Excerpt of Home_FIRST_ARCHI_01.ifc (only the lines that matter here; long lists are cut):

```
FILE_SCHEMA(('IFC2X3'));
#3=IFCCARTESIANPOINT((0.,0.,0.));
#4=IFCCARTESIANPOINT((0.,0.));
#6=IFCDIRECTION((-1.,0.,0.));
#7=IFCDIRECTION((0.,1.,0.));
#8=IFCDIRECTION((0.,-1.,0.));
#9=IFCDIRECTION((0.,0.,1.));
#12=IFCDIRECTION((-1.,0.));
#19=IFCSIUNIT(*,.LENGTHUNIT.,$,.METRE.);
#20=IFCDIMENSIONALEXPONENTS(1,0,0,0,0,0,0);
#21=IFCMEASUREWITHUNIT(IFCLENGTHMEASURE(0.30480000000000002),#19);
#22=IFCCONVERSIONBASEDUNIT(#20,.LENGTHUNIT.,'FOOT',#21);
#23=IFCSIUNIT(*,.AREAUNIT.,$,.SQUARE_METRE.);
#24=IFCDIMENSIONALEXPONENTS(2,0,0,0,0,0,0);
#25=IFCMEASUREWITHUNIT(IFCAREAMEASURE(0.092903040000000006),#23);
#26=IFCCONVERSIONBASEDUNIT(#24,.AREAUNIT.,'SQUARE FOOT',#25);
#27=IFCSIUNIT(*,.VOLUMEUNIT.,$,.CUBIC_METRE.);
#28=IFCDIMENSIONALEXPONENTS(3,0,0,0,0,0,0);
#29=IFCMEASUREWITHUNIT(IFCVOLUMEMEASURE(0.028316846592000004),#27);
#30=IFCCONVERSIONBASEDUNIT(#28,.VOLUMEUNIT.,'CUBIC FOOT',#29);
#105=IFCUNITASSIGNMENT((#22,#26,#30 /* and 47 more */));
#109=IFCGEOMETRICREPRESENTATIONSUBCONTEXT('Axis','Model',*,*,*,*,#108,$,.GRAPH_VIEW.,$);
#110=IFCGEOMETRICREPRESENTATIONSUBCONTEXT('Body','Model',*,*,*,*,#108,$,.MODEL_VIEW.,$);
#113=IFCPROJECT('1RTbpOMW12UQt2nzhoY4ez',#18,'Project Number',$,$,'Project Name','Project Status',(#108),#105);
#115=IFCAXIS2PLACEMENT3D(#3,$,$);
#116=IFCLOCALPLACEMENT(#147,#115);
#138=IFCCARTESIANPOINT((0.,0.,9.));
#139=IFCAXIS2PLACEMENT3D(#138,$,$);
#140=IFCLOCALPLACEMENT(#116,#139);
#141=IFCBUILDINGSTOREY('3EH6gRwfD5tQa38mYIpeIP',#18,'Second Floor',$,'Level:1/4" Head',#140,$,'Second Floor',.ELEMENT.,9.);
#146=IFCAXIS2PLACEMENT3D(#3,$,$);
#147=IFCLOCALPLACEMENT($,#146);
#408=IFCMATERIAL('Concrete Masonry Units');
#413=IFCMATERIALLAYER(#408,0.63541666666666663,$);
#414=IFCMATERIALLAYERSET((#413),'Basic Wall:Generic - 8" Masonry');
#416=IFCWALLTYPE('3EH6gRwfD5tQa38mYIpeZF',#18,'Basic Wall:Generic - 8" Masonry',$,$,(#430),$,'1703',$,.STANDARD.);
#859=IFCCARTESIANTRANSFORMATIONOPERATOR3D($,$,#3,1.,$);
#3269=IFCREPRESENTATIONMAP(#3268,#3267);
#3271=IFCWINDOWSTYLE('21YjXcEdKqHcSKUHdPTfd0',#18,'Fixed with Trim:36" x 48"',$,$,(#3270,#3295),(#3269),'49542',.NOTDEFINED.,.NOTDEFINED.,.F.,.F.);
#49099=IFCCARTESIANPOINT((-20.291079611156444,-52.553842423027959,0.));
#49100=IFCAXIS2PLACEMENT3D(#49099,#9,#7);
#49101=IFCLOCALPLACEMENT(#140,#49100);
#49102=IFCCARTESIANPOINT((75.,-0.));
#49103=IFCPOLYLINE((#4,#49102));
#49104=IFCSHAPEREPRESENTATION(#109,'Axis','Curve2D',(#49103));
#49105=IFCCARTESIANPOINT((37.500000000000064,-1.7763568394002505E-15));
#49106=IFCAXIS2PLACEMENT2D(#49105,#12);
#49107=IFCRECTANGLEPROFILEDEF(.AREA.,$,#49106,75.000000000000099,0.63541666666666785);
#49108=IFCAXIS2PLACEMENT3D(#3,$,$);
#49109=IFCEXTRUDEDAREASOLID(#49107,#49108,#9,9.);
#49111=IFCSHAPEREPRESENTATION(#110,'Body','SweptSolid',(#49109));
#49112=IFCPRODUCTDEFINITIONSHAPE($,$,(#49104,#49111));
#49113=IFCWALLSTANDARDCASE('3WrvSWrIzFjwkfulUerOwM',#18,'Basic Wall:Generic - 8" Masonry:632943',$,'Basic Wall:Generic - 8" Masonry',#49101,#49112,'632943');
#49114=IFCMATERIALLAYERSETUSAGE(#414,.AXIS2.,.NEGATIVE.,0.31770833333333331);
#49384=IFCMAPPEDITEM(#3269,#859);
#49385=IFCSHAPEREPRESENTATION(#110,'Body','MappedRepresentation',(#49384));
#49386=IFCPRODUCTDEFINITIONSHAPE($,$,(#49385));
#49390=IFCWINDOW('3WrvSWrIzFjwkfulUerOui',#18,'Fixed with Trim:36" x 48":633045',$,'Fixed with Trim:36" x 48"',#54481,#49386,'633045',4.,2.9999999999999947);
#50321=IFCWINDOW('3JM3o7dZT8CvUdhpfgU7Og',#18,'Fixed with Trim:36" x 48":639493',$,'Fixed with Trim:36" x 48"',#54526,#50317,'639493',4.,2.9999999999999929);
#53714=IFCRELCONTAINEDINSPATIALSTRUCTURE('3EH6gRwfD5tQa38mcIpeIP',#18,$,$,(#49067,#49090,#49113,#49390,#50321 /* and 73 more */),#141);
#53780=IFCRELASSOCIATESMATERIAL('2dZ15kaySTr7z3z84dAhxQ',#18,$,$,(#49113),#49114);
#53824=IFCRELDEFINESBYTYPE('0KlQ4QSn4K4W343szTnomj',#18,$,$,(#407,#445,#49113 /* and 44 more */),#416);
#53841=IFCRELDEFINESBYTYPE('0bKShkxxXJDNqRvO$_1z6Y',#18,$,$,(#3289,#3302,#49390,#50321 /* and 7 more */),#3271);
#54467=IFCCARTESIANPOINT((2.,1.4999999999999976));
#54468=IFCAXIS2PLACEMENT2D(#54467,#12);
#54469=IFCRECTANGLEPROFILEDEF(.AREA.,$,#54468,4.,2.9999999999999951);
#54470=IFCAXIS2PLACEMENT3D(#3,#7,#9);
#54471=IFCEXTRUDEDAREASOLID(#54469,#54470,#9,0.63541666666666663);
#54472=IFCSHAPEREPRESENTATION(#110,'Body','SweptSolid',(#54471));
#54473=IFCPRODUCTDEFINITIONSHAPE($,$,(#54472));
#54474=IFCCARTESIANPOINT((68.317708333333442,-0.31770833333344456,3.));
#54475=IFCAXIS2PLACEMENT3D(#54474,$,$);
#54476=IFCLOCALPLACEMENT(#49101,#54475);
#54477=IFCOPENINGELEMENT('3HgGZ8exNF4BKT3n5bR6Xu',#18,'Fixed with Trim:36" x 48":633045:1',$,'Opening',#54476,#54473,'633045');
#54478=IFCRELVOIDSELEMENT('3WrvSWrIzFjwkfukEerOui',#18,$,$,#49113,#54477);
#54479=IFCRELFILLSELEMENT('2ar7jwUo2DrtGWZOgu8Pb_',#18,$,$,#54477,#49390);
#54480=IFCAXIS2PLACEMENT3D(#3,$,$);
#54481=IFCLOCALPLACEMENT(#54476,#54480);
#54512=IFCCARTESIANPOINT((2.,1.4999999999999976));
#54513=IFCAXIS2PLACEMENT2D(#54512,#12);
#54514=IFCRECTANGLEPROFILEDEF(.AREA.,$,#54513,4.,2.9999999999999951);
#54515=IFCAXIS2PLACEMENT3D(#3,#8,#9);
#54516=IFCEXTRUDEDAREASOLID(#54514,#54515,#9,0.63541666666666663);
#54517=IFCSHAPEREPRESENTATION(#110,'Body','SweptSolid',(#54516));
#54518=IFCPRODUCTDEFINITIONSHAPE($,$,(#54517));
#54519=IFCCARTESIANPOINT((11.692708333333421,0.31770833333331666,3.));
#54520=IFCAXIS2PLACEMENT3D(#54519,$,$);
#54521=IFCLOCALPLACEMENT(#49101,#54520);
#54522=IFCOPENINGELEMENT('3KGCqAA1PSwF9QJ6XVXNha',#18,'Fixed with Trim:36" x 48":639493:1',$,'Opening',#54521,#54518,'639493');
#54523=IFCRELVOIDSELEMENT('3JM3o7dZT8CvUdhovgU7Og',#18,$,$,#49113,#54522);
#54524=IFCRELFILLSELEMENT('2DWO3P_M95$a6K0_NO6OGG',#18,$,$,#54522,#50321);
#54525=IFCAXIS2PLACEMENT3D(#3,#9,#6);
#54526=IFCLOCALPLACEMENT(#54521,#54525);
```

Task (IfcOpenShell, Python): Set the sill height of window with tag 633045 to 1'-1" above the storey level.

```python
import numpy as np
import ifcopenshell
import ifcopenshell.api.geometry
import ifcopenshell.geom
import ifcopenshell.util.element
import ifcopenshell.util.placement
import ifcopenshell.util.shape
import ifcopenshell.util.unit

model = ifcopenshell.open("Home_FIRST_ARCHI_01.ifc")
unit_scale = ifcopenshell.util.unit.calculate_unit_scale(model)

window = model.by_guid("3WrvSWrIzFjwkfulUerOui")
opening = window.FillsVoids[0].RelatingOpeningElement
storey = ifcopenshell.util.element.get_container(window, ifc_class="IfcBuildingStorey")
level = ifcopenshell.util.placement.get_local_placement(storey.ObjectPlacement)[2, 3]

# The opening's origin need not be at the sill, so measure its lowest point.
shape = ifcopenshell.geom.create_shape(ifcopenshell.geom.settings(), opening)
bottom = ifcopenshell.util.shape.get_shape_bottom_elevation(shape, shape.geometry) / unit_scale
dz = level + 13 * 0.0254 / unit_scale - bottom

shift = np.array([0.0, 0.0, dz])
# The window is placed relative to its opening, so it follows when the opening moves.
matrix = ifcopenshell.util.placement.get_local_placement(opening.ObjectPlacement)
matrix[:3, 3] += shift
ifcopenshell.api.geometry.edit_object_placement(
    model, product=opening, matrix=matrix, is_si=False, should_transform_children=True
)

print(f"moved by {dz * unit_scale:+.3f} m")

model.write("Home_FIRST_ARCHI_01-out.ifc")
```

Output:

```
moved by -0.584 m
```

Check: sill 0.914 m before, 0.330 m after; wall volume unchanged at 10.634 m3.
